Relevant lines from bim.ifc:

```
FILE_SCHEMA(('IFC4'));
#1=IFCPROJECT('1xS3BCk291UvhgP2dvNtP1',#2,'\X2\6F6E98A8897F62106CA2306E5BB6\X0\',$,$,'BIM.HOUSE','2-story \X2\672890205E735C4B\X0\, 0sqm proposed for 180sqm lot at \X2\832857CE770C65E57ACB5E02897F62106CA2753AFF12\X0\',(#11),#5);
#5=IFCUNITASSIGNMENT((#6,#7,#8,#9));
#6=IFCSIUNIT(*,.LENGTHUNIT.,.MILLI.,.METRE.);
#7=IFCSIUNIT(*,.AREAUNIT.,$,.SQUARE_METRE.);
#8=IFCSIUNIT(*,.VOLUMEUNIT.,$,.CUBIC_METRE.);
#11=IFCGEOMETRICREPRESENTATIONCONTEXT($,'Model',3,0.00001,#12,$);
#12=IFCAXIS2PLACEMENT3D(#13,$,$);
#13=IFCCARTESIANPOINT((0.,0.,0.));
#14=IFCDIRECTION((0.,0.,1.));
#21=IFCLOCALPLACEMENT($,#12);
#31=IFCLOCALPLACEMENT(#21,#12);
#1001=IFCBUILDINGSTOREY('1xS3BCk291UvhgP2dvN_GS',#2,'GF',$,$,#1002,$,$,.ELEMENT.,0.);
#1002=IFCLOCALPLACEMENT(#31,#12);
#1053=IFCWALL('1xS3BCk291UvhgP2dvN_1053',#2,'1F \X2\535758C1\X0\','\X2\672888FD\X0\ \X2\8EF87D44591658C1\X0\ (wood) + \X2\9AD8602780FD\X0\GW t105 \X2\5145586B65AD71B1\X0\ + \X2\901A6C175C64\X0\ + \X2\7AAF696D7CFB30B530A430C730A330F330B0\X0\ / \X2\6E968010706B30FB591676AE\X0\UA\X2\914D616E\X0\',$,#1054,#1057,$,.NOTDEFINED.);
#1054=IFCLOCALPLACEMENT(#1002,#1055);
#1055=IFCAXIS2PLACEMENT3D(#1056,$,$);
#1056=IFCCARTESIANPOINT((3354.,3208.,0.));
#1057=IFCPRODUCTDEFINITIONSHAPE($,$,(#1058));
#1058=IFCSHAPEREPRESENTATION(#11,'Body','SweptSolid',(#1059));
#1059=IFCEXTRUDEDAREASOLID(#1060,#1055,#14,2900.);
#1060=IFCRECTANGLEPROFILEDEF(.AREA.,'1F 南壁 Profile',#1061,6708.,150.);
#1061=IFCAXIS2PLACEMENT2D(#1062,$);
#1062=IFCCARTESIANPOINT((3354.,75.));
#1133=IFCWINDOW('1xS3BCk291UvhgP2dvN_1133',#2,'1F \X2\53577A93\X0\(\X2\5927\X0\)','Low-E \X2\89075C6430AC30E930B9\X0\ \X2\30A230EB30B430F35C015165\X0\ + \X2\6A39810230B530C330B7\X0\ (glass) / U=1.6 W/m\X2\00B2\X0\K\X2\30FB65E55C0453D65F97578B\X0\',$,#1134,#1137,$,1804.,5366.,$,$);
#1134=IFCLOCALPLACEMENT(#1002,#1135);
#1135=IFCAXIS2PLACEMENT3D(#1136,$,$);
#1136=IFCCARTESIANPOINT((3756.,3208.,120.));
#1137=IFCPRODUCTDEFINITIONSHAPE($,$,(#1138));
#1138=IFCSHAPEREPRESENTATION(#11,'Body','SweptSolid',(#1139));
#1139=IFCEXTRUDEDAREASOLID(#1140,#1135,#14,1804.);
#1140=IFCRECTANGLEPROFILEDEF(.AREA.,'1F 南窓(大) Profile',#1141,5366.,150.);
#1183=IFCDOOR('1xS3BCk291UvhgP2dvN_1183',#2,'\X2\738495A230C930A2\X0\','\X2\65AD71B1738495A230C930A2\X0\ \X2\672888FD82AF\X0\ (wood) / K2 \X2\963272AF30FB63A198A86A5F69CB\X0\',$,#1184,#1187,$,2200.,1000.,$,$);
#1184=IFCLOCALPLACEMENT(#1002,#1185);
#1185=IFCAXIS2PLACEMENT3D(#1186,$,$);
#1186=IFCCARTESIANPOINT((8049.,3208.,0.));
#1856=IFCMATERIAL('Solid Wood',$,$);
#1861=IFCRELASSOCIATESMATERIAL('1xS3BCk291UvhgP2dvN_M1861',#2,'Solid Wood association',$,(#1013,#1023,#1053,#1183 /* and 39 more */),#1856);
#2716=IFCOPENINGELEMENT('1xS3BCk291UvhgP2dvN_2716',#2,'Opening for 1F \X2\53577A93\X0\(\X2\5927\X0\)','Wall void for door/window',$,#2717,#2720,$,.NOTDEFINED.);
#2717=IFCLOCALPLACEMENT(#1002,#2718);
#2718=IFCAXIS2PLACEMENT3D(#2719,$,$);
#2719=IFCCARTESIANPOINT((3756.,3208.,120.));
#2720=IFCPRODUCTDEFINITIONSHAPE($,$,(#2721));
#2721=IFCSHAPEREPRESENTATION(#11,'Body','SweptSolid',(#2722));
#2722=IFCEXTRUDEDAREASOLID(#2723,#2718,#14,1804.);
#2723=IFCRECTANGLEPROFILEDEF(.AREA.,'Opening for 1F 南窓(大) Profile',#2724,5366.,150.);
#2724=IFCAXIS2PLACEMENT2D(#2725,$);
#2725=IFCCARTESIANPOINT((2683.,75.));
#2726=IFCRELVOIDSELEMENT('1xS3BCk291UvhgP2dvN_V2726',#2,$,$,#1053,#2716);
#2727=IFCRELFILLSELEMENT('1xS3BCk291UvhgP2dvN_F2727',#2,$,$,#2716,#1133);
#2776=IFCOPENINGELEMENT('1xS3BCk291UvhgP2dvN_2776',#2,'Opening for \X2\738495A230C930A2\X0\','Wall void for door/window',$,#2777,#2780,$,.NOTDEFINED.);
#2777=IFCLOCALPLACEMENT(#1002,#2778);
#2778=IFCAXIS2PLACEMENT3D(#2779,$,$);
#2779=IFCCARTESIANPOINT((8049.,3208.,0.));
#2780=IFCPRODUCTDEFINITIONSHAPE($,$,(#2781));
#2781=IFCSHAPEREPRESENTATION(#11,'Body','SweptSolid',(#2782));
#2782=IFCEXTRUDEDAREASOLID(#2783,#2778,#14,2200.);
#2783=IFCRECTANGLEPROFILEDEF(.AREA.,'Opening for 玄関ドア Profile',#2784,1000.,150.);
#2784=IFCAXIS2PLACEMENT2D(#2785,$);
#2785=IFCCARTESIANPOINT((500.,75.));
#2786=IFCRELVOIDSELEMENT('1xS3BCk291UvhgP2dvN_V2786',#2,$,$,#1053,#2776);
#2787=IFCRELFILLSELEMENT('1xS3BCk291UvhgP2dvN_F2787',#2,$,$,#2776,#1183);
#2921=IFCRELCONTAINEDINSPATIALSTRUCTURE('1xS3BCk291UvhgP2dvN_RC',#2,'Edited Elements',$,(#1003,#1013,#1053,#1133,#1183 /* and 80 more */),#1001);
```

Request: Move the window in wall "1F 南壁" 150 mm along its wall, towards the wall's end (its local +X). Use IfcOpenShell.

```python
import ifcopenshell
import ifcopenshell.api.geometry
import ifcopenshell.util.placement
import ifcopenshell.util.unit

model = ifcopenshell.open("bim.ifc")
unit_scale = ifcopenshell.util.unit.calculate_unit_scale(model)

window = model.by_guid("1xS3BCk291UvhgP2dvN_1133")
opening = window.FillsVoids[0].RelatingOpeningElement
wall = opening.VoidsElements[0].RelatingBuildingElement

wall_matrix = ifcopenshell.util.placement.get_local_placement(wall.ObjectPlacement)
shift = wall_matrix[:3, 0] * 0.15 / unit_scale
before = ifcopenshell.util.placement.get_local_placement(window.ObjectPlacement)[:3, 3].copy()

# The window is not placed relative to its opening, so move both.
for product in (opening, window):
    matrix = ifcopenshell.util.placement.get_local_placement(product.ObjectPlacement)
    matrix[:3, 3] += shift
    ifcopenshell.api.geometry.edit_object_placement(model, product=product, matrix=matrix, is_si=False)

after = ifcopenshell.util.placement.get_local_placement(window.ObjectPlacement)[:3, 3]
print("window moved by", (after - before).round(3) + 0.0)

model.write("bim_edited.ifc")
```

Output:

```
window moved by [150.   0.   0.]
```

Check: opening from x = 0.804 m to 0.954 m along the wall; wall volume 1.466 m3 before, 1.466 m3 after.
